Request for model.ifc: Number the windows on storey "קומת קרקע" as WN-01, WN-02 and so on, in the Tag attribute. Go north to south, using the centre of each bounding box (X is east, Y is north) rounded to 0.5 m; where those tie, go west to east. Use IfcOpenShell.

First a look at what the model holds.

```python
import ifcopenshell
import ifcopenshell.util.element
import ifcopenshell.util.placement

model = ifcopenshell.open("model.ifc")
print(model.schema)
storey = next(s for s in model.by_type("IfcBuildingStorey") if s.Name == "קומת קרקע")
windows = [e for e in ifcopenshell.util.element.get_decomposition(storey) if e.is_a("IfcWindow")]
for e in sorted(windows, key=lambda e: e.id()):
    origin = ifcopenshell.util.placement.get_local_placement(e.ObjectPlacement)[:3, 3]
    print(e.id(), e.Tag, e.Name, origin.round(2) + 0.0, sep=" | ")
```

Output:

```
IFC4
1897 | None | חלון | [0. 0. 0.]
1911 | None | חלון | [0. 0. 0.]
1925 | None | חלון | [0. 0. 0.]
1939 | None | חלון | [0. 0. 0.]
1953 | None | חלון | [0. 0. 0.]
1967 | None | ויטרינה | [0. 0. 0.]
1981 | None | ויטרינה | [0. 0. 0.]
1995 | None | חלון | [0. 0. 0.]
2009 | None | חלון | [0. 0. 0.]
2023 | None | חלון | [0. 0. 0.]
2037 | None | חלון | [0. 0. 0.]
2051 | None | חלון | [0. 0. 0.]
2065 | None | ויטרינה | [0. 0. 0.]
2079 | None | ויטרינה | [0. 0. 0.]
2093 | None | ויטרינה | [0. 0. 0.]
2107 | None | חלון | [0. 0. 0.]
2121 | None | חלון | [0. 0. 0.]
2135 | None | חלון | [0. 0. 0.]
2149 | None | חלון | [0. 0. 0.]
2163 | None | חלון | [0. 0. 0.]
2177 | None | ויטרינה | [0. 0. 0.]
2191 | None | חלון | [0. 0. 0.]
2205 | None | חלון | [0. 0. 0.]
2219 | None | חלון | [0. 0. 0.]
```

```python
import ifcopenshell
import ifcopenshell.geom
import ifcopenshell.util.element
import ifcopenshell.util.shape

model = ifcopenshell.open("model.ifc")
settings = ifcopenshell.geom.settings()
settings.set("use-world-coords", True)


def centre(element):
    shape = ifcopenshell.geom.create_shape(settings, element)
    return ifcopenshell.util.shape.get_bbox_centroid(shape.geometry)


storey = next(s for s in model.by_type("IfcBuildingStorey") if s.Name == "קומת קרקע")
windows = [e for e in ifcopenshell.util.element.get_decomposition(storey) if e.is_a("IfcWindow")]

# Insertion points can sit at a corner or the storey origin, so sort by the geometry (in metres).
centres = {e: centre(e) for e in windows}
windows.sort(key=lambda e: (-round(centres[e][1] / 0.5), centres[e][0]))

for i, e in enumerate(windows, start=1):
    number = f"WN-{i:02d}"
    e.Tag = number
    print(e.id(), number)

model.write("model_edited.ifc")
```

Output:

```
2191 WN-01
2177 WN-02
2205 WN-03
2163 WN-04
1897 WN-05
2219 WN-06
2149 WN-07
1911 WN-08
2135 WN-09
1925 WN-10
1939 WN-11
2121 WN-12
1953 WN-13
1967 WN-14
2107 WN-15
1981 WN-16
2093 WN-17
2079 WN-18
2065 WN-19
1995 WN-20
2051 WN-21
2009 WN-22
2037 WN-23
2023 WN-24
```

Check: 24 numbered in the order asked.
